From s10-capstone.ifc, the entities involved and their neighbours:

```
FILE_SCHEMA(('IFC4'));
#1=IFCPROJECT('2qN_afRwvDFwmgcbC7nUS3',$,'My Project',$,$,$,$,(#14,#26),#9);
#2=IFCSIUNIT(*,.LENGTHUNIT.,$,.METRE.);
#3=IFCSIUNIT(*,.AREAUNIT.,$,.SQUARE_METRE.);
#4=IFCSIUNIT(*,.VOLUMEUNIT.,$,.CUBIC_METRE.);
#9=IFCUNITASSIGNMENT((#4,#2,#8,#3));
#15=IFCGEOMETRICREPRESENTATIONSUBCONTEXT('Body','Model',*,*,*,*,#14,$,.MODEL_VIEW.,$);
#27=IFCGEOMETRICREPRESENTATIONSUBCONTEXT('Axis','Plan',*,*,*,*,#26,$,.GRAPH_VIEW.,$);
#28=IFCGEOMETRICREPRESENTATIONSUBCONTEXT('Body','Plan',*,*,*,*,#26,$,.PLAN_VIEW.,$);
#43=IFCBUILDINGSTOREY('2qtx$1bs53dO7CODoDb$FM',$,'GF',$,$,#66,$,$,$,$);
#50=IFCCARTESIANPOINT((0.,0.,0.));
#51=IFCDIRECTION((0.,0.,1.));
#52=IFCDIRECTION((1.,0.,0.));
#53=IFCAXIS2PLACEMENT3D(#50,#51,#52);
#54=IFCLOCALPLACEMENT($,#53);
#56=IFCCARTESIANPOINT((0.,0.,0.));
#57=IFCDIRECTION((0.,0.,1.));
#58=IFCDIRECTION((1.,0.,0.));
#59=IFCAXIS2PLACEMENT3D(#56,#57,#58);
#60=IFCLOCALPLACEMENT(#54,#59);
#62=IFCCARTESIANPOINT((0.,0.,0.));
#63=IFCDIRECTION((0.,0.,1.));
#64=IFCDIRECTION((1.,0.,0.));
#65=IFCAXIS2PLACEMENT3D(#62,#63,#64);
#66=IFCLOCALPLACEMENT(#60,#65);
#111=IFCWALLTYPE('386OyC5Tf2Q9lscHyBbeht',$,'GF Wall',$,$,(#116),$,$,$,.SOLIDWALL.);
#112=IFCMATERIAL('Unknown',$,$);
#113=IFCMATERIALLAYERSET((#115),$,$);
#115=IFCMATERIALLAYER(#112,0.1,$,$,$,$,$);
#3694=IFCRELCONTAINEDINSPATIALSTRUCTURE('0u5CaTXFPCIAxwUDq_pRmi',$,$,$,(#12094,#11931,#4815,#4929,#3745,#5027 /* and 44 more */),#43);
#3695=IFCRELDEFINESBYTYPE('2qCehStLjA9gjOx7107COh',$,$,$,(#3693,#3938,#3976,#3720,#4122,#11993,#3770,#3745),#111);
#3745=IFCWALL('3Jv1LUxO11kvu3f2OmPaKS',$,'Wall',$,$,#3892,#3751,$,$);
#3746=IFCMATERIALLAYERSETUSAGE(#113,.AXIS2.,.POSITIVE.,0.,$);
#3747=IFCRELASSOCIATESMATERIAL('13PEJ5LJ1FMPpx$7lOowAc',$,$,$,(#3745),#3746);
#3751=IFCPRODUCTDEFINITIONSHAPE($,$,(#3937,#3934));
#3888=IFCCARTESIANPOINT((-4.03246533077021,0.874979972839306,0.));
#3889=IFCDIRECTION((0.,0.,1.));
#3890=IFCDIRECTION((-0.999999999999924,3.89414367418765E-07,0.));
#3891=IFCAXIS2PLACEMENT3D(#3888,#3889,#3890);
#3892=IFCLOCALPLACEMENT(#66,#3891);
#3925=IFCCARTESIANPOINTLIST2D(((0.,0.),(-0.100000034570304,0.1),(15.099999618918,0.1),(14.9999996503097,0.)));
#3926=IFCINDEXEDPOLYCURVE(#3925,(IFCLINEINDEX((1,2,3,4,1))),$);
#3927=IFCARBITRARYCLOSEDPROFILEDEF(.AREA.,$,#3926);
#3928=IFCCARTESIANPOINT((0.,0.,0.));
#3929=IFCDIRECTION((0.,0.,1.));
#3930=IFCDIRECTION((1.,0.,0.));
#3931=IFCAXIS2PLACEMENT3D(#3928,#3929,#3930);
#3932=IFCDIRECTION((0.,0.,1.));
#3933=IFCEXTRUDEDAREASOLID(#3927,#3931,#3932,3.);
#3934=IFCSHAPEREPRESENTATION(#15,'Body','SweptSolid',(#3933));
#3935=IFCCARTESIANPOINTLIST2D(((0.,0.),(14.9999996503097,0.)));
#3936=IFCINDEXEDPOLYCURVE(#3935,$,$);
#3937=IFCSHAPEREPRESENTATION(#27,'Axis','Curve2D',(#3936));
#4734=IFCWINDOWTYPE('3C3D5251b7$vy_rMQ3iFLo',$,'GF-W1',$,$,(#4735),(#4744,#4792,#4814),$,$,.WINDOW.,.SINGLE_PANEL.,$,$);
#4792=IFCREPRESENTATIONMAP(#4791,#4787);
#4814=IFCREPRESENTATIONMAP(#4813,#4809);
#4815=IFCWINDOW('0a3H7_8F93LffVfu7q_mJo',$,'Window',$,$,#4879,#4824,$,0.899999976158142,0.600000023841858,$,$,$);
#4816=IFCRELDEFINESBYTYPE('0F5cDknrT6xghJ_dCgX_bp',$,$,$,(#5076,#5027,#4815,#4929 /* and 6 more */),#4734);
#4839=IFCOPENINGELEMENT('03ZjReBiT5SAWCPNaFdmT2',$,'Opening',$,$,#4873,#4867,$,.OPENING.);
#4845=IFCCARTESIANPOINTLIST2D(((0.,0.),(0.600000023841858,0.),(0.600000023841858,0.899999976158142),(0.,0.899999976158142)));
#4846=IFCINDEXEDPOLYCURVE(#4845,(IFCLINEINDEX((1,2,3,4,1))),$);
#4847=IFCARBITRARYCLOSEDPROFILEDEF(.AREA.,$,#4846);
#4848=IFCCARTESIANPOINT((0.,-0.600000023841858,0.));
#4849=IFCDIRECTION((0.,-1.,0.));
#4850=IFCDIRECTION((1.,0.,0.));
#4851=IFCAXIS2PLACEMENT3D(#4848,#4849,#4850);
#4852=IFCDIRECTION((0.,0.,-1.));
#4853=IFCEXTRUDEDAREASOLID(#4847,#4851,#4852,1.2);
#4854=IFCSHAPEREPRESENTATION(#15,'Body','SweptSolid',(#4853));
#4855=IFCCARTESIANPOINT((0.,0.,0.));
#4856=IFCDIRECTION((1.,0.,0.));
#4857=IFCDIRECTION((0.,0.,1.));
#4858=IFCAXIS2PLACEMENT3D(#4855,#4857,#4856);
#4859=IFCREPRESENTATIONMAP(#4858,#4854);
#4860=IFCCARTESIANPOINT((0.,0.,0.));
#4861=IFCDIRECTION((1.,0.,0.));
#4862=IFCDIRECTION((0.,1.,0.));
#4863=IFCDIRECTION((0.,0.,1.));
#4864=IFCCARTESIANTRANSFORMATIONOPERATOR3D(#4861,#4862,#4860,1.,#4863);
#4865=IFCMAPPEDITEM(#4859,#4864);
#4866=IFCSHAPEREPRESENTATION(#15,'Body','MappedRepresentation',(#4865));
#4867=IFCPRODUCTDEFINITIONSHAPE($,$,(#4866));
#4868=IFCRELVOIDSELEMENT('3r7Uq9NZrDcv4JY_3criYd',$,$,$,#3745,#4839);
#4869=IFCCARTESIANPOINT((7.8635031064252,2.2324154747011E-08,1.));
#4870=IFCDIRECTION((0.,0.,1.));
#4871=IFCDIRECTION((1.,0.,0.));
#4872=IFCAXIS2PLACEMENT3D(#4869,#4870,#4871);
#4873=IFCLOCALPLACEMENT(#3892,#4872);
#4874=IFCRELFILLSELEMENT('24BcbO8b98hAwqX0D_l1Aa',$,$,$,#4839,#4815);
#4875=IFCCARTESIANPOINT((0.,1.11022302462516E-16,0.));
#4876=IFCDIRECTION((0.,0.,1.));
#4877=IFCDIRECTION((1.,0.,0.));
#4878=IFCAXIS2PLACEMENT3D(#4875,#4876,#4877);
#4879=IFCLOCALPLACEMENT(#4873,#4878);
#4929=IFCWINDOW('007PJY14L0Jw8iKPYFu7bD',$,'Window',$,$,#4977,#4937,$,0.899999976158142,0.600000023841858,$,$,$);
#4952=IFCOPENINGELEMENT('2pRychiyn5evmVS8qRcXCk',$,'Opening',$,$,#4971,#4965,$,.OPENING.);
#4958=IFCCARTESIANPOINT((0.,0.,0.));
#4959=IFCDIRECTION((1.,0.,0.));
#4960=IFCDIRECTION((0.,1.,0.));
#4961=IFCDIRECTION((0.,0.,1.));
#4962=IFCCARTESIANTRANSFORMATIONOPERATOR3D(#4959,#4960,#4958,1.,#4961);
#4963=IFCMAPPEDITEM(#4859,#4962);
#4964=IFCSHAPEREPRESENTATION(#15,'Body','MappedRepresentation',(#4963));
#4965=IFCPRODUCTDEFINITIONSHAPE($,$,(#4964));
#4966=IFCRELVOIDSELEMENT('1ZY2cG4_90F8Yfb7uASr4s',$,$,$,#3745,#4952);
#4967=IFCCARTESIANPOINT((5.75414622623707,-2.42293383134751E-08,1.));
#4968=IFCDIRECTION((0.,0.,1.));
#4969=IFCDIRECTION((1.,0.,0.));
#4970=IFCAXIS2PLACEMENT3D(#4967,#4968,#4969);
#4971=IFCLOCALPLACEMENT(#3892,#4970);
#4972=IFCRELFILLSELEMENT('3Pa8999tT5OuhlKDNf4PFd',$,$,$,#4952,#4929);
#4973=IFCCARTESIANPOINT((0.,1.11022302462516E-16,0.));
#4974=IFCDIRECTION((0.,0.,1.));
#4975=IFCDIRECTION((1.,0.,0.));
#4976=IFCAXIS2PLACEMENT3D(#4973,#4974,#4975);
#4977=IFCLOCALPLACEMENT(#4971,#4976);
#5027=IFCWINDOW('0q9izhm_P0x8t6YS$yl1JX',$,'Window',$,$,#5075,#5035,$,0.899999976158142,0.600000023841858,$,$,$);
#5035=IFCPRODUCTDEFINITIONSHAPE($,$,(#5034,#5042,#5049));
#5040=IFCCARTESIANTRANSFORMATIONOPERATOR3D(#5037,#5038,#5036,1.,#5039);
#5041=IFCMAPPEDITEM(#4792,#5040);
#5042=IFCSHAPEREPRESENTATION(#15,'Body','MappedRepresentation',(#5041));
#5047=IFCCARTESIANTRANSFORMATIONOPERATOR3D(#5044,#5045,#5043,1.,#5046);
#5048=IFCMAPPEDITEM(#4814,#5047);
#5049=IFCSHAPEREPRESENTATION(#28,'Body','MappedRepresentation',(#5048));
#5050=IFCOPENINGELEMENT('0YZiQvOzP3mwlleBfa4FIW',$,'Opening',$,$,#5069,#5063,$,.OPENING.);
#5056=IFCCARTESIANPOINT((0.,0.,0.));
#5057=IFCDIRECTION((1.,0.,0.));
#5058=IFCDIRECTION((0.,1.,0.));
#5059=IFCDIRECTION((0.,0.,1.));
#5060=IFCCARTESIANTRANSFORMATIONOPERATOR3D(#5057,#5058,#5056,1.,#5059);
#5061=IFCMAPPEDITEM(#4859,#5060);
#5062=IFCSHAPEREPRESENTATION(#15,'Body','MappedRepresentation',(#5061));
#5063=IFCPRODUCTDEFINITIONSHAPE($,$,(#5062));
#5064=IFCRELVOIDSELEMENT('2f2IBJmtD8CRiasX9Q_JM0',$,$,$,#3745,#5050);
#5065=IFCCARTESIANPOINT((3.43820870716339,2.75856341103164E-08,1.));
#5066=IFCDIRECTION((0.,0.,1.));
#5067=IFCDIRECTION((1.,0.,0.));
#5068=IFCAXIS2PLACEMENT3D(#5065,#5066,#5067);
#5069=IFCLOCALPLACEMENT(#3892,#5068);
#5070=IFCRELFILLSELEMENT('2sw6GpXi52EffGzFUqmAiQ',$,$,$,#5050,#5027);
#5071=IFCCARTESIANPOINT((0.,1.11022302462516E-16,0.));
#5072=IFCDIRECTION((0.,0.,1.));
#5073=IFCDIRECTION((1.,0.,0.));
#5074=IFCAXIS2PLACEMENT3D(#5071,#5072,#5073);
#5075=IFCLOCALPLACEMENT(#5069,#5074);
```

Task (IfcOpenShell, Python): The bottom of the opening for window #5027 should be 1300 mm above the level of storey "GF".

```python
import numpy as np
import ifcopenshell
import ifcopenshell.api.geometry
import ifcopenshell.geom
import ifcopenshell.util.element
import ifcopenshell.util.placement
import ifcopenshell.util.shape
import ifcopenshell.util.unit

model = ifcopenshell.open("s10-capstone.ifc")
unit_scale = ifcopenshell.util.unit.calculate_unit_scale(model)

window = model.by_id(5027)
opening = window.FillsVoids[0].RelatingOpeningElement
storey = ifcopenshell.util.element.get_container(window, ifc_class="IfcBuildingStorey")
level = ifcopenshell.util.placement.get_local_placement(storey.ObjectPlacement)[2, 3]

# The opening's origin need not be at the sill, so measure its lowest point.
shape = ifcopenshell.geom.create_shape(ifcopenshell.geom.settings(), opening)
bottom = ifcopenshell.util.shape.get_shape_bottom_elevation(shape, shape.geometry) / unit_scale
dz = level + 1.3 / unit_scale - bottom

shift = np.array([0.0, 0.0, dz])
# The window is placed relative to its opening, so it follows when the opening moves.
matrix = ifcopenshell.util.placement.get_local_placement(opening.ObjectPlacement)
matrix[:3, 3] += shift
ifcopenshell.api.geometry.edit_object_placement(
    model, product=opening, matrix=matrix, is_si=False, should_transform_children=True
)

print(f"moved by {dz * unit_scale:+.3f} m")

model.write("s10-capstone_rev.ifc")
```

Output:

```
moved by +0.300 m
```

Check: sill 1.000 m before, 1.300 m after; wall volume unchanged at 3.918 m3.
